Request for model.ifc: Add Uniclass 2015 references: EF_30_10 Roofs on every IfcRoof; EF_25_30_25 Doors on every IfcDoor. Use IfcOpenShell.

First a look at what the model holds.

```python
import ifcopenshell

model = ifcopenshell.open("model.ifc")
print(model.schema)
print("classifications:", [c.Name for c in model.by_type("IfcClassification")])
for ifc_class in ("IfcDoor", "IfcRoof", "IfcStair", "IfcWall", "IfcWindow"):
    print(ifc_class, len(model.by_type(ifc_class)))
```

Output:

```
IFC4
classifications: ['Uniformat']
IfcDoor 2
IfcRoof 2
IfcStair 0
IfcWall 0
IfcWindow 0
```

```python
import ifcopenshell
import ifcopenshell.api.classification

model = ifcopenshell.open("model.ifc")

system = ifcopenshell.api.classification.add_classification(model, classification="Uniclass 2015")

codes = {
    "IfcRoof": ("EF_30_10", "Roofs"),
    "IfcDoor": ("EF_25_30_25", "Doors"),
}
for ifc_class, (code, name) in codes.items():
    products = model.by_type(ifc_class)
    ifcopenshell.api.classification.add_reference(
        model, products=products, classification=system, identification=code, name=name
    )
    print(code, len(products))

model.write("model_updated.ifc")
```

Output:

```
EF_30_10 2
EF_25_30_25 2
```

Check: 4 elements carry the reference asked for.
